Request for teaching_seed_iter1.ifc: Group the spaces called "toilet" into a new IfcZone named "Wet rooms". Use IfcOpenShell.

First a look at what the model holds.

```python
import ifcopenshell

model = ifcopenshell.open("teaching_seed_iter1.ifc")
print(model.schema)
seen = {}
for space in model.by_type("IfcSpace"):
    seen[space.LongName] = seen.get(space.LongName, 0) + 1
for name, count in sorted(seen.items(), key=str):
    print(count, "x", name)
print("zones:", [z.Name for z in model.by_type("IfcZone")][:20])
```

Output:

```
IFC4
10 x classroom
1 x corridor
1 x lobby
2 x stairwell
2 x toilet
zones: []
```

```python
import ifcopenshell
import ifcopenshell.api.group
import ifcopenshell.api.root

model = ifcopenshell.open("teaching_seed_iter1.ifc")

names = {"toilet"}
spaces = [s for s in model.by_type("IfcSpace") if s.LongName in names]

zone = ifcopenshell.api.root.create_entity(model, ifc_class="IfcZone", name="Wet rooms")
ifcopenshell.api.group.assign_group(model, products=spaces, group=zone)
print(len(spaces), "spaces in", zone.Name)

model.write("teaching_seed_iter1_rev.ifc")
```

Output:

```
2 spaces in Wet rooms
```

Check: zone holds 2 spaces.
